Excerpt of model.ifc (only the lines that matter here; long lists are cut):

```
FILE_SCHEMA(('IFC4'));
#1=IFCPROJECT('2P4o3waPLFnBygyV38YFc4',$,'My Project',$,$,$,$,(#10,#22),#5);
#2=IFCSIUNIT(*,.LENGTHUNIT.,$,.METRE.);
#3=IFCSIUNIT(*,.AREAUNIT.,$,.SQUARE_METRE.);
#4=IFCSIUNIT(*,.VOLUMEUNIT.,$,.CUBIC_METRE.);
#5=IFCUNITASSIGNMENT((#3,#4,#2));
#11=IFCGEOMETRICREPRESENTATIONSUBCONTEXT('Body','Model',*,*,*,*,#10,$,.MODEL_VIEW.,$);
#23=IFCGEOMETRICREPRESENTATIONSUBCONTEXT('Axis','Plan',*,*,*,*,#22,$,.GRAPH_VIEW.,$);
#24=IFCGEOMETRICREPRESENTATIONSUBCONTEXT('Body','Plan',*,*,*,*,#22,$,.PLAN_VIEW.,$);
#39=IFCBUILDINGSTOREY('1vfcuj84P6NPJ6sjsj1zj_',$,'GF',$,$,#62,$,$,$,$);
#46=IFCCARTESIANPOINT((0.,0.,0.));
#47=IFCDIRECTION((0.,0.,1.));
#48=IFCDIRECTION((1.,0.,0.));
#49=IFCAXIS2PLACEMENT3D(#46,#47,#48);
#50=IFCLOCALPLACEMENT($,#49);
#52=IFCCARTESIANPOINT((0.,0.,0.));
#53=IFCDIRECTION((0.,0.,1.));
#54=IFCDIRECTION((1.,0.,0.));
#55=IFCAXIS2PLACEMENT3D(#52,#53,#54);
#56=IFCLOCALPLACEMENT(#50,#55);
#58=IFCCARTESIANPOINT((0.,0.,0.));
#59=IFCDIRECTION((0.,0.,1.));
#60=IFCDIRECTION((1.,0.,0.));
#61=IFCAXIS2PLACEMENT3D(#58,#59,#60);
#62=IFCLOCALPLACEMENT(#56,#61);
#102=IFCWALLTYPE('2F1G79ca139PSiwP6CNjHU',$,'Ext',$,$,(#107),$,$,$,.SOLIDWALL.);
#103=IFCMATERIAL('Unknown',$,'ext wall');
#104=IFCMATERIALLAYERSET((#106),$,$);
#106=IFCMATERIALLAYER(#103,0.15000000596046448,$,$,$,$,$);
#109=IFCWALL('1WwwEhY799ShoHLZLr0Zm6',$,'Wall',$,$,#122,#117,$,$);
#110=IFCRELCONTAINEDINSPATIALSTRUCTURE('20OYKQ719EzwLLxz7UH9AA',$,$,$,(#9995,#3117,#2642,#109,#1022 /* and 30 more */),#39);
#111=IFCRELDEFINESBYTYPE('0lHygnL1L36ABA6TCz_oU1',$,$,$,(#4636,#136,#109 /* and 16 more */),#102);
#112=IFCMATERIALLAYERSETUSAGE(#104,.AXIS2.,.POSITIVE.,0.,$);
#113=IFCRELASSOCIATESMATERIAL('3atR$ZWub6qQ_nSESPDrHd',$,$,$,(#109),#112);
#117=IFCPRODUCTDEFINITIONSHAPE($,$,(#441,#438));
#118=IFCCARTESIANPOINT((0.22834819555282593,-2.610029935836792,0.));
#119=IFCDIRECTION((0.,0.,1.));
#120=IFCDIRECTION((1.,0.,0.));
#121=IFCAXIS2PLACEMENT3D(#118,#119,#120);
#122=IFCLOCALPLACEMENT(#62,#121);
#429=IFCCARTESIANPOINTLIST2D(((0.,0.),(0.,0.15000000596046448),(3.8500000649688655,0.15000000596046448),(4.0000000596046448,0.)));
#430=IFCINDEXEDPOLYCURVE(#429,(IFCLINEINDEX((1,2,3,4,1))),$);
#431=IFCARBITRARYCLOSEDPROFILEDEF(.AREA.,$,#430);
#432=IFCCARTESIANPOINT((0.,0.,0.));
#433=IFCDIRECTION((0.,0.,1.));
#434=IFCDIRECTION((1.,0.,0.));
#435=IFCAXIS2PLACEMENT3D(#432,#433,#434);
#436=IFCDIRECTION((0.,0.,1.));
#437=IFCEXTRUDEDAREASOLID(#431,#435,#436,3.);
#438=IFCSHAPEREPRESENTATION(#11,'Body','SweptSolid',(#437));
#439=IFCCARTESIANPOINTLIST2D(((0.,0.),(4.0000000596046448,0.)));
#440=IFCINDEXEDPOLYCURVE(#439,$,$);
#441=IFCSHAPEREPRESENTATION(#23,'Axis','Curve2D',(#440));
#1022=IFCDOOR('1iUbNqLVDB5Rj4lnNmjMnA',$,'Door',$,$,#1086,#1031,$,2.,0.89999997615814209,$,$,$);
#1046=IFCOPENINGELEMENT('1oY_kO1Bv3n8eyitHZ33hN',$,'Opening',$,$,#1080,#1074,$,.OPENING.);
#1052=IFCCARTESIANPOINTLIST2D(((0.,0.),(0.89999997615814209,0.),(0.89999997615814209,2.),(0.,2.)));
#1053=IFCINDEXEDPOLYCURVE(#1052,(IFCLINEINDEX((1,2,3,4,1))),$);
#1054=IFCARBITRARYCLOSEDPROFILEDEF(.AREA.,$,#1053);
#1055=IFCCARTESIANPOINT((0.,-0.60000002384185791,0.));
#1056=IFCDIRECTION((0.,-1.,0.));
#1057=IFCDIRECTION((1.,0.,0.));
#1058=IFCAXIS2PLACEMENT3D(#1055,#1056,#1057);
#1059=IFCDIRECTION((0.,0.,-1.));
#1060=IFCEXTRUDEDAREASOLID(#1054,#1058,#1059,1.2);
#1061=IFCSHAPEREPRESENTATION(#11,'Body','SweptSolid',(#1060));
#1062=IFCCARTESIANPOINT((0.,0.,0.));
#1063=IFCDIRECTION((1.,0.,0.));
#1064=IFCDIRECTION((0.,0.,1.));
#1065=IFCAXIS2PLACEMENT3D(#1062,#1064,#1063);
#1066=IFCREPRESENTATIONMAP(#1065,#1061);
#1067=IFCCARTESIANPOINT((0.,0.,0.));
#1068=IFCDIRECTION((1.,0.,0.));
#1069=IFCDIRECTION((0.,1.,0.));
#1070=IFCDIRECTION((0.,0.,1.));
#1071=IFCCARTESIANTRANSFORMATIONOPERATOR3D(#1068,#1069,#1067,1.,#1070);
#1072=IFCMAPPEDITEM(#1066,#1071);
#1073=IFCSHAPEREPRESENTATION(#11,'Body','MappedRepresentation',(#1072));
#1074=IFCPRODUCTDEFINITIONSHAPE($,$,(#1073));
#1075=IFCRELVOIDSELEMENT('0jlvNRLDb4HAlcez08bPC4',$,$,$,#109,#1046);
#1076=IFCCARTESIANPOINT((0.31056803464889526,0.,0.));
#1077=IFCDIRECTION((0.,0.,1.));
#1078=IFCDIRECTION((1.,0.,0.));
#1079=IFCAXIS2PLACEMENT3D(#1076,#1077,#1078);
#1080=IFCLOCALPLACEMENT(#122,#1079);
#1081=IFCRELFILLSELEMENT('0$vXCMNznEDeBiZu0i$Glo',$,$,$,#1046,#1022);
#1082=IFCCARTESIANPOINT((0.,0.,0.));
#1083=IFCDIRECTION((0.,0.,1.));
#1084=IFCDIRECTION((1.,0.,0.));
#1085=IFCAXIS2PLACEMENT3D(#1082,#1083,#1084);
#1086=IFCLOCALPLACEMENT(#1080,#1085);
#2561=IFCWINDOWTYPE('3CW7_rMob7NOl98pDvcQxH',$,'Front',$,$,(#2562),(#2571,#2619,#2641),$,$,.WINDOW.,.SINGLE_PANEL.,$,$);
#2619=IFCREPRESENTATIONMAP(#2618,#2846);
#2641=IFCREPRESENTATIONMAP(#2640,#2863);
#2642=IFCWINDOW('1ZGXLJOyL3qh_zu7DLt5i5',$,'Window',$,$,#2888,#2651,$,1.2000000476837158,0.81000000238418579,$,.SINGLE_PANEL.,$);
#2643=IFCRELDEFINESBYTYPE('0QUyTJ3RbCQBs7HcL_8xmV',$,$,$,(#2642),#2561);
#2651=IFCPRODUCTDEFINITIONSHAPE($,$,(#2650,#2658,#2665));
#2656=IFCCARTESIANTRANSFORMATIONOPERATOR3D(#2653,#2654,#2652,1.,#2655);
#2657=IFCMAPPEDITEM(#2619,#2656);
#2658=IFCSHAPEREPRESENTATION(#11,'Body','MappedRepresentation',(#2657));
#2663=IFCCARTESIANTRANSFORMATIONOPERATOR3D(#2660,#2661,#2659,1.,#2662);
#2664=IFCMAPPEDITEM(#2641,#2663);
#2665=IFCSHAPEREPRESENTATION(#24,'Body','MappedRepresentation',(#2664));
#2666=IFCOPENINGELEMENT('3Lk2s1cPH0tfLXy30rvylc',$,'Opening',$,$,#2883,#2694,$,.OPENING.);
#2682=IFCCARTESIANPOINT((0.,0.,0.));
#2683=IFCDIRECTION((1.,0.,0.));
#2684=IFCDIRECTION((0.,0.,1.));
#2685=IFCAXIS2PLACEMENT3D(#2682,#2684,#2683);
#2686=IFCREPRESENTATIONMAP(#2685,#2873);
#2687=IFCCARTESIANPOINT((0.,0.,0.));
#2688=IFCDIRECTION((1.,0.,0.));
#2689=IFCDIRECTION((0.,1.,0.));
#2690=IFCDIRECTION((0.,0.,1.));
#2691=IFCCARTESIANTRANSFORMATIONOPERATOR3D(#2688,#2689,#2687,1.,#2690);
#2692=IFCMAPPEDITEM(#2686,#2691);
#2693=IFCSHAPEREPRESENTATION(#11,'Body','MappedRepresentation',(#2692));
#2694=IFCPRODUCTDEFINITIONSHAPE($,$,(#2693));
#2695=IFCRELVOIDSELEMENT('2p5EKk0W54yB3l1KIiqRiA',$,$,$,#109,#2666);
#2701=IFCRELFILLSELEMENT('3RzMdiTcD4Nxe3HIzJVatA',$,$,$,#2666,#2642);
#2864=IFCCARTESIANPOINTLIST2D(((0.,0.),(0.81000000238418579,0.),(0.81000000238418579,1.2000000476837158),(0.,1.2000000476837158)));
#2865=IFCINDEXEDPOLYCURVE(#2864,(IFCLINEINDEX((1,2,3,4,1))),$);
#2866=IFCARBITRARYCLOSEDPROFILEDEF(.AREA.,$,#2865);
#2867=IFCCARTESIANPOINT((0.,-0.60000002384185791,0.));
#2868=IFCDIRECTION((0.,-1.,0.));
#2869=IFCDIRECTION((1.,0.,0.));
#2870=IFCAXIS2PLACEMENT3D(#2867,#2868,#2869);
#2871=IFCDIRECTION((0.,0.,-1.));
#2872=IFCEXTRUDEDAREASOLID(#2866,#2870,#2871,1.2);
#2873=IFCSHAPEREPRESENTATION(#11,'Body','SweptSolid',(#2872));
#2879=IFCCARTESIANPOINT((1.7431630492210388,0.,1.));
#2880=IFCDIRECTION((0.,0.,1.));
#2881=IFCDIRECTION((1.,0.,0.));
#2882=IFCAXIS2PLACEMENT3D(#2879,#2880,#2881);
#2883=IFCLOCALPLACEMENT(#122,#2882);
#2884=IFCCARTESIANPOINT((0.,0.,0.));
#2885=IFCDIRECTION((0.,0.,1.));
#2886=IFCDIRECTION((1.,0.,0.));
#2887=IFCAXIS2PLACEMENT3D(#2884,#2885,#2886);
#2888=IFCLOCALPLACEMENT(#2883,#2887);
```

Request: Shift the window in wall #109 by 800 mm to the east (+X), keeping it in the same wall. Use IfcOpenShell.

```python
import ifcopenshell
import ifcopenshell.api.geometry
import ifcopenshell.util.placement

model = ifcopenshell.open("model.ifc")

window = model.by_guid("1ZGXLJOyL3qh_zu7DLt5i5")
opening = window.FillsVoids[0].RelatingOpeningElement
wall = opening.VoidsElements[0].RelatingBuildingElement

wall_matrix = ifcopenshell.util.placement.get_local_placement(wall.ObjectPlacement)
shift = wall_matrix[:3, 0] * 0.8
before = ifcopenshell.util.placement.get_local_placement(window.ObjectPlacement)[:3, 3].copy()

# The window is placed relative to its opening, so it follows when the opening moves.
matrix = ifcopenshell.util.placement.get_local_placement(opening.ObjectPlacement)
matrix[:3, 3] += shift
ifcopenshell.api.geometry.edit_object_placement(
    model, product=opening, matrix=matrix, is_si=False, should_transform_children=True
)

after = ifcopenshell.util.placement.get_local_placement(window.ObjectPlacement)[:3, 3]
print("window moved by", (after - before).round(3) + 0.0)

model.write("model-out.ifc")
```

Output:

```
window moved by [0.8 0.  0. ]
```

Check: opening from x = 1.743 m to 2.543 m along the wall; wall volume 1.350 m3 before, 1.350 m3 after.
